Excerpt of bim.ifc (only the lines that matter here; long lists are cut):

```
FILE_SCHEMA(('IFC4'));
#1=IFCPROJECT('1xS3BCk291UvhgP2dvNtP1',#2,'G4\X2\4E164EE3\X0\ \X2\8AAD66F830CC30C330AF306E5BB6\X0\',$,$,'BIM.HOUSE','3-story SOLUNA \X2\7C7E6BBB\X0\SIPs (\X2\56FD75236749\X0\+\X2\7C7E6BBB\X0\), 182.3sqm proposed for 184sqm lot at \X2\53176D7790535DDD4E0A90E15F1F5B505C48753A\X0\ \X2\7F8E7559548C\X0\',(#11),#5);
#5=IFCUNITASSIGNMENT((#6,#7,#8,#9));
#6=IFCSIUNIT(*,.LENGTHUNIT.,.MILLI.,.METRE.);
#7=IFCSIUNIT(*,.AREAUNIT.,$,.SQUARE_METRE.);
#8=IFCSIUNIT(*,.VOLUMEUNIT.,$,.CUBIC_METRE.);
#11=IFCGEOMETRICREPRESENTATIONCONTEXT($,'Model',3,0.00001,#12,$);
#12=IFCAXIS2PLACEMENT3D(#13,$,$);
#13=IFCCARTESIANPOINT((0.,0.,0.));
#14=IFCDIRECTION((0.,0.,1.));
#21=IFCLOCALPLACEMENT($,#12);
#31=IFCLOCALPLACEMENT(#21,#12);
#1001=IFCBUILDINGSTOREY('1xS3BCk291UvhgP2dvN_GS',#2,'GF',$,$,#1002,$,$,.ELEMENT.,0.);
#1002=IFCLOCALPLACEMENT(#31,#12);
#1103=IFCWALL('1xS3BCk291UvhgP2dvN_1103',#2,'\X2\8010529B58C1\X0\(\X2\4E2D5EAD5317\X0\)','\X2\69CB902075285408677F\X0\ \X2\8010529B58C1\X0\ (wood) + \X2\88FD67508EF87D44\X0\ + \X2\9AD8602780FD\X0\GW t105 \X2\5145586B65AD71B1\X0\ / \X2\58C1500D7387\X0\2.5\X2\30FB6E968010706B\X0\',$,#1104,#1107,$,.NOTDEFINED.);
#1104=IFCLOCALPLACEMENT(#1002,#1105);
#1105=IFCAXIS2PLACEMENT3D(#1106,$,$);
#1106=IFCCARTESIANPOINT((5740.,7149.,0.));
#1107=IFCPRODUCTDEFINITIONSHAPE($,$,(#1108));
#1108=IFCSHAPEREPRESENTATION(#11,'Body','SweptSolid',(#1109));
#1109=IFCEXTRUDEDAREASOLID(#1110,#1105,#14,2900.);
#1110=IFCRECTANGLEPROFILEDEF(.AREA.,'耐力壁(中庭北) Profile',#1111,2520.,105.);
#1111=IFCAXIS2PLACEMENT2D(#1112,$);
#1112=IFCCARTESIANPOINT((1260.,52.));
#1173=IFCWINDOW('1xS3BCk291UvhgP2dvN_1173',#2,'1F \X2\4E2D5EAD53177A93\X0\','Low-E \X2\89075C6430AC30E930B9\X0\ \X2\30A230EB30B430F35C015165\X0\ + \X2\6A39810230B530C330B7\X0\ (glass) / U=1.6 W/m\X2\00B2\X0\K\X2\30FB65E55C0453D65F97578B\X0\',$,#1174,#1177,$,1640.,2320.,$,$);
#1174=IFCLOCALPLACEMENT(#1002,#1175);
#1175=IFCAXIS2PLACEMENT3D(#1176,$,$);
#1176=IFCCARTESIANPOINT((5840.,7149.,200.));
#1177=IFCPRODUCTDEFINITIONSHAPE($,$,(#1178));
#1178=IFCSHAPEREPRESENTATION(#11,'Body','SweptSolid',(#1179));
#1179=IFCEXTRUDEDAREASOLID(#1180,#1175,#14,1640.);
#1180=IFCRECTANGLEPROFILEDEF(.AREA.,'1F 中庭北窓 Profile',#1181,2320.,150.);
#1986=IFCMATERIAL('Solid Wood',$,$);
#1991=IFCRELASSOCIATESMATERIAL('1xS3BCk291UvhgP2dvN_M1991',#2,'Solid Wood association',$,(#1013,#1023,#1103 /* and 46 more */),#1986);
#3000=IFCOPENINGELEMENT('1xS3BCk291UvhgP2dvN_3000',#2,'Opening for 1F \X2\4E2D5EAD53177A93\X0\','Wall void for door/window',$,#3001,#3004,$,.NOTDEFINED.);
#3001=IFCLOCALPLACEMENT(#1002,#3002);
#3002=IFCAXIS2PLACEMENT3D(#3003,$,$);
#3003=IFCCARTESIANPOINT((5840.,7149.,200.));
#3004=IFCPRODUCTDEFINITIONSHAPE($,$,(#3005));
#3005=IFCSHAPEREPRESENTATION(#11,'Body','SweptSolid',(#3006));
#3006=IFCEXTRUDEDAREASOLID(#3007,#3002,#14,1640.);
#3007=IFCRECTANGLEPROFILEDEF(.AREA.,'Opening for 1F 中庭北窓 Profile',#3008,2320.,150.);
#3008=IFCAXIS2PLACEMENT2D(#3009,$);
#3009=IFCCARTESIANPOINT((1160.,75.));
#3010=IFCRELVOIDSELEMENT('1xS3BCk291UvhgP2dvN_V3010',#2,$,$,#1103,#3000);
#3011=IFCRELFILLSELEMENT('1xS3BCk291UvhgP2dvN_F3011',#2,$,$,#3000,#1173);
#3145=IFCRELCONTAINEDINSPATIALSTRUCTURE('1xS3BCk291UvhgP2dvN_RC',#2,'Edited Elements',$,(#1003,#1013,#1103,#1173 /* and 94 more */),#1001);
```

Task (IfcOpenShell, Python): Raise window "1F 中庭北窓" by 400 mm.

```python
import numpy as np
import ifcopenshell
import ifcopenshell.api.geometry
import ifcopenshell.util.placement
import ifcopenshell.util.unit

model = ifcopenshell.open("bim.ifc")
unit_scale = ifcopenshell.util.unit.calculate_unit_scale(model)

window = model.by_id(1173)
opening = window.FillsVoids[0].RelatingOpeningElement
dz = 0.4 / unit_scale

shift = np.array([0.0, 0.0, dz])
# The window is not placed relative to its opening, so move both.
for product in (opening, window):
    matrix = ifcopenshell.util.placement.get_local_placement(product.ObjectPlacement)
    matrix[:3, 3] += shift
    ifcopenshell.api.geometry.edit_object_placement(model, product=product, matrix=matrix, is_si=False)

print(f"moved by {dz * unit_scale:+.3f} m")

model.write("bim_rev.ifc")
```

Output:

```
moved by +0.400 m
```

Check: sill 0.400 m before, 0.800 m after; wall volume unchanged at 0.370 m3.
